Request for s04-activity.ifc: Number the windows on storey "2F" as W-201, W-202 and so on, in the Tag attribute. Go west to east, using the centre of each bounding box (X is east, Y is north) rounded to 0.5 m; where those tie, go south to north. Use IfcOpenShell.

First a look at what the model holds.

```python
import ifcopenshell
import ifcopenshell.util.element
import ifcopenshell.util.placement

model = ifcopenshell.open("s04-activity.ifc")
print(model.schema)
storey = next(s for s in model.by_type("IfcBuildingStorey") if s.Name == "2F")
windows = [e for e in ifcopenshell.util.element.get_decomposition(storey) if e.is_a("IfcWindow")]
for e in sorted(windows, key=lambda e: e.id()):
    origin = ifcopenshell.util.placement.get_local_placement(e.ObjectPlacement)[:3, 3]
    print(e.id(), e.Tag, e.Name, origin.round(2) + 0.0, sep=" | ")
```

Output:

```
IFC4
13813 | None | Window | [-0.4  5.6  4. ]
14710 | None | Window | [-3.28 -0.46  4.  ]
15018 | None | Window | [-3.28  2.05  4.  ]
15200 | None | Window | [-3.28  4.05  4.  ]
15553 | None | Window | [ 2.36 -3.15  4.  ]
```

```python
import ifcopenshell
import ifcopenshell.geom
import ifcopenshell.util.element
import ifcopenshell.util.shape

model = ifcopenshell.open("s04-activity.ifc")
settings = ifcopenshell.geom.settings()
settings.set("use-world-coords", True)


def centre(element):
    shape = ifcopenshell.geom.create_shape(settings, element)
    return ifcopenshell.util.shape.get_bbox_centroid(shape.geometry)


storey = next(s for s in model.by_type("IfcBuildingStorey") if s.Name == "2F")
windows = [e for e in ifcopenshell.util.element.get_decomposition(storey) if e.is_a("IfcWindow")]

# Insertion points can sit at a corner or the storey origin, so sort by the geometry (in metres).
centres = {e: centre(e) for e in windows}
windows.sort(key=lambda e: (round(centres[e][0] / 0.5), centres[e][1]))

for i, e in enumerate(windows, start=1):
    number = f"W-2{i:02d}"
    e.Tag = number
    print(e.id(), number)

model.write("s04-activity_rev.ifc")
```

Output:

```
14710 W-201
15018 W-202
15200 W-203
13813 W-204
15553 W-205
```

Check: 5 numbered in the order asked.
